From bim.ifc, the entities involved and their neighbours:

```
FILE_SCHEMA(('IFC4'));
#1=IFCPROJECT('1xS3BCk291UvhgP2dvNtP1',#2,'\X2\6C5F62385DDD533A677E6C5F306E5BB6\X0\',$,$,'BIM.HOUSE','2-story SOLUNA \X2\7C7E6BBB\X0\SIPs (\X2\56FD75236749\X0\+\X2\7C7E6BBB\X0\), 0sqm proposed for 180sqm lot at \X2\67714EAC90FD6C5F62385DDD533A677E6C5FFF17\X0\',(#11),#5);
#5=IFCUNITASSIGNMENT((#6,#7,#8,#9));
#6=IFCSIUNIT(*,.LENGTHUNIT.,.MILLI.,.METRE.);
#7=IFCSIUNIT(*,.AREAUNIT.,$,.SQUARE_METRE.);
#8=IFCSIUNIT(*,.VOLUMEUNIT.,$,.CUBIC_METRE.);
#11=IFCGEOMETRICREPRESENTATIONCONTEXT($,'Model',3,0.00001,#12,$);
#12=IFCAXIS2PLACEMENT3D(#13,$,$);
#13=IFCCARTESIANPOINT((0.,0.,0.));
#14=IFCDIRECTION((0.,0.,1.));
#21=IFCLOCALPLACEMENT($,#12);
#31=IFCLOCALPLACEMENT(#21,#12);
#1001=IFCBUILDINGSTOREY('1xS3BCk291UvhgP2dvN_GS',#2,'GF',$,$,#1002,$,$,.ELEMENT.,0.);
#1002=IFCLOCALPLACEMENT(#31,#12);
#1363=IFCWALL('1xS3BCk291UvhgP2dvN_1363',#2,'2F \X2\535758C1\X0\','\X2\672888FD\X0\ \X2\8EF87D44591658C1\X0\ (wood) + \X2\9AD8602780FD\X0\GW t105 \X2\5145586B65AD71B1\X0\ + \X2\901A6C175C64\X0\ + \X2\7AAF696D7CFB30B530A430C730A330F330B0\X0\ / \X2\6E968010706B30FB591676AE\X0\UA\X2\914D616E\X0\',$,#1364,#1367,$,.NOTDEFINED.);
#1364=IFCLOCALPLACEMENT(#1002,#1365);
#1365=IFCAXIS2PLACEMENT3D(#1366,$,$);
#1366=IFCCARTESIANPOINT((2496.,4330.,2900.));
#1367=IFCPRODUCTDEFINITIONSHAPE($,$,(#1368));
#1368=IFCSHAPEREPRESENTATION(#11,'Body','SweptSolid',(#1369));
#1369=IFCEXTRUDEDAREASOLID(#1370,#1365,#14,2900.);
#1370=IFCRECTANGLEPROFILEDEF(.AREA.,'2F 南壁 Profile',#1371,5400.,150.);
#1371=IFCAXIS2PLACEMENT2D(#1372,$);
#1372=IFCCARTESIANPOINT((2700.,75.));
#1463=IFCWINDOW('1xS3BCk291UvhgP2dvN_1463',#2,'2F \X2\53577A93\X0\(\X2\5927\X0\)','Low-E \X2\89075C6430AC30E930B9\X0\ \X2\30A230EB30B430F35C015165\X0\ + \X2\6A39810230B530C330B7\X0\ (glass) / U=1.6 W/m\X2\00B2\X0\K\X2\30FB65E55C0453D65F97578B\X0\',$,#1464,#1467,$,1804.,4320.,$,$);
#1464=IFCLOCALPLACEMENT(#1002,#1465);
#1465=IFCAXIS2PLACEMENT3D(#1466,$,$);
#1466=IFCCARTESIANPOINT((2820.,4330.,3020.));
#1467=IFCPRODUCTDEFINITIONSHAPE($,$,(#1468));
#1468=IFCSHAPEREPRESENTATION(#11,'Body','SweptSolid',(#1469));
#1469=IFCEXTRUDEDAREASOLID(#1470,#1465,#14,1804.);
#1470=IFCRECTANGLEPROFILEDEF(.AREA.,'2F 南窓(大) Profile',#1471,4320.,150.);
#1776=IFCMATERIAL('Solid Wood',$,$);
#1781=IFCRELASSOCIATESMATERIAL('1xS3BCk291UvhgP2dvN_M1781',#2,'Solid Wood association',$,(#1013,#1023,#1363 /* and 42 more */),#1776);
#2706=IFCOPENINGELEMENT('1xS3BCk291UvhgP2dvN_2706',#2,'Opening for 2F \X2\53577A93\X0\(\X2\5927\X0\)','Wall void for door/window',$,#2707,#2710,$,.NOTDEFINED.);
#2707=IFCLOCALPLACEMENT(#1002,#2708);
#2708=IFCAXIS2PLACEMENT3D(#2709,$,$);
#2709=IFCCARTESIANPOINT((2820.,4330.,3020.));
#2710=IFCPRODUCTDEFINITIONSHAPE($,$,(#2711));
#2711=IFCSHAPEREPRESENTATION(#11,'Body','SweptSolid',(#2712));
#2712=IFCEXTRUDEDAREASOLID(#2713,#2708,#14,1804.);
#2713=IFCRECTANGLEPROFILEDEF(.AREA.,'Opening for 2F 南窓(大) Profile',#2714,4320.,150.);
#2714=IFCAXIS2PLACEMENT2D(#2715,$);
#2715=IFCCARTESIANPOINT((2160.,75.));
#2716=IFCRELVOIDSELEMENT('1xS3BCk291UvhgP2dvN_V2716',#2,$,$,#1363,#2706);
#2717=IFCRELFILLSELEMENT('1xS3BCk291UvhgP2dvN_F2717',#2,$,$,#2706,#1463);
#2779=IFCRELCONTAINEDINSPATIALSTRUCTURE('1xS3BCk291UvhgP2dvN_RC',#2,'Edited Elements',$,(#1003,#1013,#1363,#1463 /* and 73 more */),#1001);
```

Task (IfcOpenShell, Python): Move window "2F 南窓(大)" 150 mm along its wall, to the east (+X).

```python
import ifcopenshell
import ifcopenshell.api.geometry
import ifcopenshell.util.placement

model = ifcopenshell.open("bim.ifc")

window = model.by_guid("1xS3BCk291UvhgP2dvN_1463")
opening = window.FillsVoids[0].RelatingOpeningElement
wall = opening.VoidsElements[0].RelatingBuildingElement

wall_matrix = ifcopenshell.util.placement.get_local_placement(wall.ObjectPlacement)
shift = wall_matrix[:3, 0] * 150.0
before = ifcopenshell.util.placement.get_local_placement(window.ObjectPlacement)[:3, 3].copy()

# The window is not placed relative to its opening, so move both.
for product in (opening, window):
    matrix = ifcopenshell.util.placement.get_local_placement(product.ObjectPlacement)
    matrix[:3, 3] += shift
    ifcopenshell.api.geometry.edit_object_placement(model, product=product, matrix=matrix, is_si=False)

after = ifcopenshell.util.placement.get_local_placement(window.ObjectPlacement)[:3, 3]
print("window moved by", (after - before).round(3) + 0.0)

model.write("bim_updated.ifc")
```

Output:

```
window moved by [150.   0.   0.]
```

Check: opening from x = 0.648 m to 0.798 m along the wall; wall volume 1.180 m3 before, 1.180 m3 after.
